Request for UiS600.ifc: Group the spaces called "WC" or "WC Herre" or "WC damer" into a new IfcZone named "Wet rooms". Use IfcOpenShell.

First a look at what the model holds.

```python
import ifcopenshell

model = ifcopenshell.open("UiS600.ifc")
print(model.schema)
seen = {}
for space in model.by_type("IfcSpace"):
    seen[space.LongName] = seen.get(space.LongName, 0) + 1
for name, count in sorted(seen.items(), key=str):
    print(count, "x", name)
print("zones:", [z.Name for z in model.by_type("IfcZone")][:20])
```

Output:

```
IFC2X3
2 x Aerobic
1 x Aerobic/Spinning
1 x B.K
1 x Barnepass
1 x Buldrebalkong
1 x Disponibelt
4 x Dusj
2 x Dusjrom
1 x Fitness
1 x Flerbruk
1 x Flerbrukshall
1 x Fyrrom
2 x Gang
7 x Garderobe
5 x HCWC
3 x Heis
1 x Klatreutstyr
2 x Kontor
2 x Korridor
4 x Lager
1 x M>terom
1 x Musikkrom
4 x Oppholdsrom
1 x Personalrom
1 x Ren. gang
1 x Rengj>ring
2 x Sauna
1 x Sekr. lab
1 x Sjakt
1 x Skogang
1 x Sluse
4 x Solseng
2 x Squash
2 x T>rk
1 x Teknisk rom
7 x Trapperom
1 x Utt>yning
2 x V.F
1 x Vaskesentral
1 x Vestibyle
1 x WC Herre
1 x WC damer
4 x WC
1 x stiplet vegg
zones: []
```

```python
import ifcopenshell
import ifcopenshell.api.group
import ifcopenshell.api.root

model = ifcopenshell.open("UiS600.ifc")

names = {"WC", "WC Herre", "WC damer"}
spaces = [s for s in model.by_type("IfcSpace") if s.LongName in names]

zone = ifcopenshell.api.root.create_entity(model, ifc_class="IfcZone", name="Wet rooms")
ifcopenshell.api.group.assign_group(model, products=spaces, group=zone)
print(len(spaces), "spaces in", zone.Name)

model.write("UiS600_edited.ifc")
```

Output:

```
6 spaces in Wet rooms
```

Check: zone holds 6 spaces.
